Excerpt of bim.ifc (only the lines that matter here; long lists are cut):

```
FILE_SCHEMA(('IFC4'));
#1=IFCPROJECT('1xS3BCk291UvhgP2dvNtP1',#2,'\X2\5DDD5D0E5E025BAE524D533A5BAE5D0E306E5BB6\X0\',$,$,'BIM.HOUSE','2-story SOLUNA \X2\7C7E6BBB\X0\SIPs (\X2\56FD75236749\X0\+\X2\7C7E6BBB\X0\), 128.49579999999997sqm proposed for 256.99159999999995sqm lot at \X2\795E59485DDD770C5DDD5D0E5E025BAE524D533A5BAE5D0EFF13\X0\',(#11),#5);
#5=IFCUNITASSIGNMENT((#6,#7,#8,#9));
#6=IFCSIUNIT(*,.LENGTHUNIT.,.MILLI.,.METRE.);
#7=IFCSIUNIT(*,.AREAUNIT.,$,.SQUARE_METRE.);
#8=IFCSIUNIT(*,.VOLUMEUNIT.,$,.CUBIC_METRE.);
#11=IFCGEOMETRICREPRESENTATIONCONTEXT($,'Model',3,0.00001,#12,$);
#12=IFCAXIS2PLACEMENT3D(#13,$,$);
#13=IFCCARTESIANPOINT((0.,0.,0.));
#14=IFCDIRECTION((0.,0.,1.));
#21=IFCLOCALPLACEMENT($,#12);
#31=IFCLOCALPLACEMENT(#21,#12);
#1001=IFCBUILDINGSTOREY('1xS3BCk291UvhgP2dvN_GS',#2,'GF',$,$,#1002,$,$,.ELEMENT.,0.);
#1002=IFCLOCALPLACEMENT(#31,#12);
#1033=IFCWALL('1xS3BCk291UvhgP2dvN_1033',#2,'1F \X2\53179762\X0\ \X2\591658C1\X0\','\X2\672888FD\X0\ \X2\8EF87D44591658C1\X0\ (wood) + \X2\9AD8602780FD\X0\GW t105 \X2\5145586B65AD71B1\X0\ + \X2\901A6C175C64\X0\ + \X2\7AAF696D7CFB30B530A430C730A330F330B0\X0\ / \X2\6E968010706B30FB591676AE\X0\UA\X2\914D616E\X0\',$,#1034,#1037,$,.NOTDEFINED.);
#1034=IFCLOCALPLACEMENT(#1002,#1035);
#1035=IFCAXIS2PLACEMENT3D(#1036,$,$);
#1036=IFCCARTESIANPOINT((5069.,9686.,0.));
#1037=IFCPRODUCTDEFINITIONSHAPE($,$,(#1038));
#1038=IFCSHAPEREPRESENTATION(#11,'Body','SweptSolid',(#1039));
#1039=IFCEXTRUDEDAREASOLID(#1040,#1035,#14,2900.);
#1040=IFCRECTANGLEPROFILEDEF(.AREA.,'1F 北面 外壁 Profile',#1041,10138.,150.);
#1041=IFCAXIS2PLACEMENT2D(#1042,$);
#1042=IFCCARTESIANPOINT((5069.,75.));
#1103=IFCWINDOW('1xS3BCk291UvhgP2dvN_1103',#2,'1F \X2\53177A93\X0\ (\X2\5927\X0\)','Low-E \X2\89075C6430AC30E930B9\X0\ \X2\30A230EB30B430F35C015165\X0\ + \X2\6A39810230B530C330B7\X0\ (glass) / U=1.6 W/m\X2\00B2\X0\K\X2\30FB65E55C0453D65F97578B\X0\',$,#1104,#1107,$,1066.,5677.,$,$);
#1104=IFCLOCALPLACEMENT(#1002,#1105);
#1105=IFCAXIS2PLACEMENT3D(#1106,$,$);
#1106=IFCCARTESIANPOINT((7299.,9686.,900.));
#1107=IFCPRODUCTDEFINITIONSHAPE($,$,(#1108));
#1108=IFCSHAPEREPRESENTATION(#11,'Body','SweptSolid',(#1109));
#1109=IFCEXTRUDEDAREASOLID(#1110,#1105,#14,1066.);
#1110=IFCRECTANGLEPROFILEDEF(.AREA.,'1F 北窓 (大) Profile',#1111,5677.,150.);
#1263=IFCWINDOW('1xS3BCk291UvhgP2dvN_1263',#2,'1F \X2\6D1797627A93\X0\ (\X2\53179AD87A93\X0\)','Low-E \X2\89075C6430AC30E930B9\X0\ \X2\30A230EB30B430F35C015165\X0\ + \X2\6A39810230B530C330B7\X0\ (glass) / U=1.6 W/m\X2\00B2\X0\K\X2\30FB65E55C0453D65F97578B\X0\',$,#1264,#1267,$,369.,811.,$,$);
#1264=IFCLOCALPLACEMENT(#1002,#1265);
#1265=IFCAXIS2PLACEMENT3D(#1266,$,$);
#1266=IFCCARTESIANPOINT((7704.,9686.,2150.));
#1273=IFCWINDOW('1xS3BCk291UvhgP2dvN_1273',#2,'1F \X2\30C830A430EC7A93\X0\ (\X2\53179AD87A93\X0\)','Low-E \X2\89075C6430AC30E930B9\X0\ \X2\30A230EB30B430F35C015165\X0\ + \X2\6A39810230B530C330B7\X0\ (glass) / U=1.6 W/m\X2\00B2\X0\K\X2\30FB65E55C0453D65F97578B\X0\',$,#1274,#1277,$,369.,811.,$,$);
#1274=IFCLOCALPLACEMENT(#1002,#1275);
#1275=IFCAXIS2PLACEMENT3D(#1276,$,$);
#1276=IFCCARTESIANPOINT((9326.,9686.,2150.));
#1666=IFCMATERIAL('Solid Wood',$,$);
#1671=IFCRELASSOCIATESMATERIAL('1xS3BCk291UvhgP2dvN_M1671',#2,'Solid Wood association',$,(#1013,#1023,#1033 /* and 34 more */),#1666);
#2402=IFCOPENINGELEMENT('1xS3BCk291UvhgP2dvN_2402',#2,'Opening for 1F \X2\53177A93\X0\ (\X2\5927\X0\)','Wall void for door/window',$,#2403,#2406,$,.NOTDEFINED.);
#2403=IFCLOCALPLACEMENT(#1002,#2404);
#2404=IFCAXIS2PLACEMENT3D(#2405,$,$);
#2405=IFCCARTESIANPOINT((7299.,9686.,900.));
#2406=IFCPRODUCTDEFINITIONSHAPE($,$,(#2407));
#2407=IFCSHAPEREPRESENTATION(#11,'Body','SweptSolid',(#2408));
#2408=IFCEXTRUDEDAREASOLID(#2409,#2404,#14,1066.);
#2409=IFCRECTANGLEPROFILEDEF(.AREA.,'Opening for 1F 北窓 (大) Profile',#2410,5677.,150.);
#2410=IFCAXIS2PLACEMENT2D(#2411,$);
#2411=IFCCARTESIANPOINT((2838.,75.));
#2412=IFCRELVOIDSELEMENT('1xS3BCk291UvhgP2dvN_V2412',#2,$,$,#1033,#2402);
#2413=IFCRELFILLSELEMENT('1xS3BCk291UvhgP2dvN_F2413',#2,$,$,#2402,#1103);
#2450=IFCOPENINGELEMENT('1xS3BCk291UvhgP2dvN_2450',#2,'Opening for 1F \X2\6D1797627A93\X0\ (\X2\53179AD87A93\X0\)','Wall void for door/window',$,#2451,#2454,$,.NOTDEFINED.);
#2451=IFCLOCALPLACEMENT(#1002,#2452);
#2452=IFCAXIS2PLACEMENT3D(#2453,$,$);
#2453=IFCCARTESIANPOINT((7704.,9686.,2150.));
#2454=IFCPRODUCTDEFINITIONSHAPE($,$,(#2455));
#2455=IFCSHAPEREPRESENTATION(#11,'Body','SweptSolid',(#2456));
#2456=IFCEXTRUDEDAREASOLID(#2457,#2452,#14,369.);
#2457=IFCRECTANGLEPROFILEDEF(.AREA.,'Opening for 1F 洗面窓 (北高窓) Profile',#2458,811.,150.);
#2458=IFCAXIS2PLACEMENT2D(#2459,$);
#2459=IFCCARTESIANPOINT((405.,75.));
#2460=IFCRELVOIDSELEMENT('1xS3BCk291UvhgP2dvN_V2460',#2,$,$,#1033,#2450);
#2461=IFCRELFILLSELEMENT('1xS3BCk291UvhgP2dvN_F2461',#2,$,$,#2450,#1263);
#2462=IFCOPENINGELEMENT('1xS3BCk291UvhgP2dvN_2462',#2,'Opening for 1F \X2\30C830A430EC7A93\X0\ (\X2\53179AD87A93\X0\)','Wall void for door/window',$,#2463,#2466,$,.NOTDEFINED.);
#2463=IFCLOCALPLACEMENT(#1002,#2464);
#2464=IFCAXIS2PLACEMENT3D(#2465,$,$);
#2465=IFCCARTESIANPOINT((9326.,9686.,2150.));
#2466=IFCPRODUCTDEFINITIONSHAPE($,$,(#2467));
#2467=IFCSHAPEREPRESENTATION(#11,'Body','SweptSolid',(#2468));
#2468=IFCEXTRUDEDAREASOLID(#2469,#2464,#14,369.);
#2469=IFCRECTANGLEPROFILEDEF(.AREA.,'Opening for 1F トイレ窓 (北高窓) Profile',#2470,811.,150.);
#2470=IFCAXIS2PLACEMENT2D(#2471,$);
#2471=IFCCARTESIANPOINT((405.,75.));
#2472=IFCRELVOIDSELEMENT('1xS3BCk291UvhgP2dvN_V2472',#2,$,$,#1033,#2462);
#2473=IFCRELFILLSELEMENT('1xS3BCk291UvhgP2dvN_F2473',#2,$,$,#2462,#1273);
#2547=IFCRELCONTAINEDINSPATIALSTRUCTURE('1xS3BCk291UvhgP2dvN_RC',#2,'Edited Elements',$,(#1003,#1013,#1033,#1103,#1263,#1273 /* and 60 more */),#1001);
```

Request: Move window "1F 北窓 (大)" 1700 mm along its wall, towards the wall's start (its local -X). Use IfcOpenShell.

```python
import ifcopenshell
import ifcopenshell.api.geometry
import ifcopenshell.util.placement
import ifcopenshell.util.unit

model = ifcopenshell.open("bim.ifc")
unit_scale = ifcopenshell.util.unit.calculate_unit_scale(model)

window = model.by_id(1103)
opening = window.FillsVoids[0].RelatingOpeningElement
wall = opening.VoidsElements[0].RelatingBuildingElement

wall_matrix = ifcopenshell.util.placement.get_local_placement(wall.ObjectPlacement)
shift = wall_matrix[:3, 0] * -1.7 / unit_scale
before = ifcopenshell.util.placement.get_local_placement(window.ObjectPlacement)[:3, 3].copy()

# The window is not placed relative to its opening, so move both.
for product in (opening, window):
    matrix = ifcopenshell.util.placement.get_local_placement(product.ObjectPlacement)
    matrix[:3, 3] += shift
    ifcopenshell.api.geometry.edit_object_placement(model, product=product, matrix=matrix, is_si=False)

after = ifcopenshell.util.placement.get_local_placement(window.ObjectPlacement)[:3, 3]
print("window moved by", (after - before).round(3) + 0.0)

model.write("bim_v2.ifc")
```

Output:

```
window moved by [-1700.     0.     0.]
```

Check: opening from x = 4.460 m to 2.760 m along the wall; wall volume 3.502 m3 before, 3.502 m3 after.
